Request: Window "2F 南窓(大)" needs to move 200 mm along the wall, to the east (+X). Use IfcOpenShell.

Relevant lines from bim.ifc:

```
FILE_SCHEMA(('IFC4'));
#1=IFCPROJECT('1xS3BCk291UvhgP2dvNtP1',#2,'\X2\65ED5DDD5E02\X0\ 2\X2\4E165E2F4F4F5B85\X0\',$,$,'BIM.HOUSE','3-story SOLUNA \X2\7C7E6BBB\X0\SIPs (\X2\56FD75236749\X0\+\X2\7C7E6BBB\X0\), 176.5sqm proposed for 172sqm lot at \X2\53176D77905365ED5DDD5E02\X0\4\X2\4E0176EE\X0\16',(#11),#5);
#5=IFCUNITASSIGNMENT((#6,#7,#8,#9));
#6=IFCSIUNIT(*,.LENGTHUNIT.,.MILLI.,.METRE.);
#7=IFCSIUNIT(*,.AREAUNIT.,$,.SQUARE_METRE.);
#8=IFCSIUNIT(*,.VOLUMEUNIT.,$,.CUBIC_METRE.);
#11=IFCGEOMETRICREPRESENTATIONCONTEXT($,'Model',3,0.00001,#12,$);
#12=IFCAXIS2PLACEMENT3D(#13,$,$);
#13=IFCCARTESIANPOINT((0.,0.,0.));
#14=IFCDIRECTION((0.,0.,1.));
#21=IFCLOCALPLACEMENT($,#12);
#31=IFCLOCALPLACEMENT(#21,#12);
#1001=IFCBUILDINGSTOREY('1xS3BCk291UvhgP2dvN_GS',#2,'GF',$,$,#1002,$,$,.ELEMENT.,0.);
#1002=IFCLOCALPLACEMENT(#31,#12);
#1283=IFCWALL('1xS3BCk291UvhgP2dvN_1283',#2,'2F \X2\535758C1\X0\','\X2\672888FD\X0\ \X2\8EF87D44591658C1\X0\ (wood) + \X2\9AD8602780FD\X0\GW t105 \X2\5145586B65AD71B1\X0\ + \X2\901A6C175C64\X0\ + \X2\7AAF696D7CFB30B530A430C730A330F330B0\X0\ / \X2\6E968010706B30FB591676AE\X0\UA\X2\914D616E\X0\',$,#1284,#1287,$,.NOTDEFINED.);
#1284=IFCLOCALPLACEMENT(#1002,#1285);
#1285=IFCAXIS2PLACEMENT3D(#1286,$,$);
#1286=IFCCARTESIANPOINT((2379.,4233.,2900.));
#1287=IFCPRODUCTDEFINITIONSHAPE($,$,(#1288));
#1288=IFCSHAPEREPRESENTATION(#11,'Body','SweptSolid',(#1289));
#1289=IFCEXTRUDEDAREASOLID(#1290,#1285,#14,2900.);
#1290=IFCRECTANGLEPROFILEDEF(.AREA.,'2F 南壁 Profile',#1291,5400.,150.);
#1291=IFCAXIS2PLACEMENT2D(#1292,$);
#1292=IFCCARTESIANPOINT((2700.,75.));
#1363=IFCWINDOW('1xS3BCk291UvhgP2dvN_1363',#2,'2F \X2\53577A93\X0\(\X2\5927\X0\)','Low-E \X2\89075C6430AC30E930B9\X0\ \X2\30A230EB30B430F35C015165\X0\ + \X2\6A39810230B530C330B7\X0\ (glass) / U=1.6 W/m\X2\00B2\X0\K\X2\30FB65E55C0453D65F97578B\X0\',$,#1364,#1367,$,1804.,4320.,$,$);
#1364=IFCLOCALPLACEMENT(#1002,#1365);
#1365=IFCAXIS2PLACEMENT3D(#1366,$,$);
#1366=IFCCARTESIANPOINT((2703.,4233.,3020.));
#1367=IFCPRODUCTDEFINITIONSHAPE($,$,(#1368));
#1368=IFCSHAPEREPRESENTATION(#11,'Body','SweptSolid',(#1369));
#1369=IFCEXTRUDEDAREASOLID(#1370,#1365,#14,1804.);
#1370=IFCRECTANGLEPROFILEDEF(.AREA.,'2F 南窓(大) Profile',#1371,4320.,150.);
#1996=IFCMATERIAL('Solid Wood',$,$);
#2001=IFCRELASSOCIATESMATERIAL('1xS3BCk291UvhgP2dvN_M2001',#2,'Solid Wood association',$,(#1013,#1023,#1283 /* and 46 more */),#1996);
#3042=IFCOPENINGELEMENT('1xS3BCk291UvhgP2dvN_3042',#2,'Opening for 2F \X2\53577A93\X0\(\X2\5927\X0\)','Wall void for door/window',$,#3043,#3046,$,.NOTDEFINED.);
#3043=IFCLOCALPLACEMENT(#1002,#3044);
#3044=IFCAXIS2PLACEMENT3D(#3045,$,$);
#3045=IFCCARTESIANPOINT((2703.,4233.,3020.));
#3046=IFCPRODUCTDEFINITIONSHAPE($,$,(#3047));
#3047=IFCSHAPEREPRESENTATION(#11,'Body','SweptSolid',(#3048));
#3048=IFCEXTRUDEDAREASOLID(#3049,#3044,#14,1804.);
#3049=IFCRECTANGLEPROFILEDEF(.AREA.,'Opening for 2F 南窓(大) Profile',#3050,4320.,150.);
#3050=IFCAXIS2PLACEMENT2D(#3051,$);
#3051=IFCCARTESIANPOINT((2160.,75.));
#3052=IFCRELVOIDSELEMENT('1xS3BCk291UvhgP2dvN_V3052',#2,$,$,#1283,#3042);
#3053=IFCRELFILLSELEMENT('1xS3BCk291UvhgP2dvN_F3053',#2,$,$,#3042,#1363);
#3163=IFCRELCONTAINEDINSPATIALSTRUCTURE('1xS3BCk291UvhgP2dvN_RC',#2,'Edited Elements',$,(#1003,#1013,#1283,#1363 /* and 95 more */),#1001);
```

```python
import ifcopenshell
import ifcopenshell.api.geometry
import ifcopenshell.util.placement
import ifcopenshell.util.unit

model = ifcopenshell.open("bim.ifc")
unit_scale = ifcopenshell.util.unit.calculate_unit_scale(model)

window = model.by_id(1363)
opening = window.FillsVoids[0].RelatingOpeningElement
wall = opening.VoidsElements[0].RelatingBuildingElement

wall_matrix = ifcopenshell.util.placement.get_local_placement(wall.ObjectPlacement)
shift = wall_matrix[:3, 0] * 0.2 / unit_scale
before = ifcopenshell.util.placement.get_local_placement(window.ObjectPlacement)[:3, 3].copy()

# The window is not placed relative to its opening, so move both.
for product in (opening, window):
    matrix = ifcopenshell.util.placement.get_local_placement(product.ObjectPlacement)
    matrix[:3, 3] += shift
    ifcopenshell.api.geometry.edit_object_placement(model, product=product, matrix=matrix, is_si=False)

after = ifcopenshell.util.placement.get_local_placement(window.ObjectPlacement)[:3, 3]
print("window moved by", (after - before).round(3) + 0.0)

model.write("bim-out.ifc")
```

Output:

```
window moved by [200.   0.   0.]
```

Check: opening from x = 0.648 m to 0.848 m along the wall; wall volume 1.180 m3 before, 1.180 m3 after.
